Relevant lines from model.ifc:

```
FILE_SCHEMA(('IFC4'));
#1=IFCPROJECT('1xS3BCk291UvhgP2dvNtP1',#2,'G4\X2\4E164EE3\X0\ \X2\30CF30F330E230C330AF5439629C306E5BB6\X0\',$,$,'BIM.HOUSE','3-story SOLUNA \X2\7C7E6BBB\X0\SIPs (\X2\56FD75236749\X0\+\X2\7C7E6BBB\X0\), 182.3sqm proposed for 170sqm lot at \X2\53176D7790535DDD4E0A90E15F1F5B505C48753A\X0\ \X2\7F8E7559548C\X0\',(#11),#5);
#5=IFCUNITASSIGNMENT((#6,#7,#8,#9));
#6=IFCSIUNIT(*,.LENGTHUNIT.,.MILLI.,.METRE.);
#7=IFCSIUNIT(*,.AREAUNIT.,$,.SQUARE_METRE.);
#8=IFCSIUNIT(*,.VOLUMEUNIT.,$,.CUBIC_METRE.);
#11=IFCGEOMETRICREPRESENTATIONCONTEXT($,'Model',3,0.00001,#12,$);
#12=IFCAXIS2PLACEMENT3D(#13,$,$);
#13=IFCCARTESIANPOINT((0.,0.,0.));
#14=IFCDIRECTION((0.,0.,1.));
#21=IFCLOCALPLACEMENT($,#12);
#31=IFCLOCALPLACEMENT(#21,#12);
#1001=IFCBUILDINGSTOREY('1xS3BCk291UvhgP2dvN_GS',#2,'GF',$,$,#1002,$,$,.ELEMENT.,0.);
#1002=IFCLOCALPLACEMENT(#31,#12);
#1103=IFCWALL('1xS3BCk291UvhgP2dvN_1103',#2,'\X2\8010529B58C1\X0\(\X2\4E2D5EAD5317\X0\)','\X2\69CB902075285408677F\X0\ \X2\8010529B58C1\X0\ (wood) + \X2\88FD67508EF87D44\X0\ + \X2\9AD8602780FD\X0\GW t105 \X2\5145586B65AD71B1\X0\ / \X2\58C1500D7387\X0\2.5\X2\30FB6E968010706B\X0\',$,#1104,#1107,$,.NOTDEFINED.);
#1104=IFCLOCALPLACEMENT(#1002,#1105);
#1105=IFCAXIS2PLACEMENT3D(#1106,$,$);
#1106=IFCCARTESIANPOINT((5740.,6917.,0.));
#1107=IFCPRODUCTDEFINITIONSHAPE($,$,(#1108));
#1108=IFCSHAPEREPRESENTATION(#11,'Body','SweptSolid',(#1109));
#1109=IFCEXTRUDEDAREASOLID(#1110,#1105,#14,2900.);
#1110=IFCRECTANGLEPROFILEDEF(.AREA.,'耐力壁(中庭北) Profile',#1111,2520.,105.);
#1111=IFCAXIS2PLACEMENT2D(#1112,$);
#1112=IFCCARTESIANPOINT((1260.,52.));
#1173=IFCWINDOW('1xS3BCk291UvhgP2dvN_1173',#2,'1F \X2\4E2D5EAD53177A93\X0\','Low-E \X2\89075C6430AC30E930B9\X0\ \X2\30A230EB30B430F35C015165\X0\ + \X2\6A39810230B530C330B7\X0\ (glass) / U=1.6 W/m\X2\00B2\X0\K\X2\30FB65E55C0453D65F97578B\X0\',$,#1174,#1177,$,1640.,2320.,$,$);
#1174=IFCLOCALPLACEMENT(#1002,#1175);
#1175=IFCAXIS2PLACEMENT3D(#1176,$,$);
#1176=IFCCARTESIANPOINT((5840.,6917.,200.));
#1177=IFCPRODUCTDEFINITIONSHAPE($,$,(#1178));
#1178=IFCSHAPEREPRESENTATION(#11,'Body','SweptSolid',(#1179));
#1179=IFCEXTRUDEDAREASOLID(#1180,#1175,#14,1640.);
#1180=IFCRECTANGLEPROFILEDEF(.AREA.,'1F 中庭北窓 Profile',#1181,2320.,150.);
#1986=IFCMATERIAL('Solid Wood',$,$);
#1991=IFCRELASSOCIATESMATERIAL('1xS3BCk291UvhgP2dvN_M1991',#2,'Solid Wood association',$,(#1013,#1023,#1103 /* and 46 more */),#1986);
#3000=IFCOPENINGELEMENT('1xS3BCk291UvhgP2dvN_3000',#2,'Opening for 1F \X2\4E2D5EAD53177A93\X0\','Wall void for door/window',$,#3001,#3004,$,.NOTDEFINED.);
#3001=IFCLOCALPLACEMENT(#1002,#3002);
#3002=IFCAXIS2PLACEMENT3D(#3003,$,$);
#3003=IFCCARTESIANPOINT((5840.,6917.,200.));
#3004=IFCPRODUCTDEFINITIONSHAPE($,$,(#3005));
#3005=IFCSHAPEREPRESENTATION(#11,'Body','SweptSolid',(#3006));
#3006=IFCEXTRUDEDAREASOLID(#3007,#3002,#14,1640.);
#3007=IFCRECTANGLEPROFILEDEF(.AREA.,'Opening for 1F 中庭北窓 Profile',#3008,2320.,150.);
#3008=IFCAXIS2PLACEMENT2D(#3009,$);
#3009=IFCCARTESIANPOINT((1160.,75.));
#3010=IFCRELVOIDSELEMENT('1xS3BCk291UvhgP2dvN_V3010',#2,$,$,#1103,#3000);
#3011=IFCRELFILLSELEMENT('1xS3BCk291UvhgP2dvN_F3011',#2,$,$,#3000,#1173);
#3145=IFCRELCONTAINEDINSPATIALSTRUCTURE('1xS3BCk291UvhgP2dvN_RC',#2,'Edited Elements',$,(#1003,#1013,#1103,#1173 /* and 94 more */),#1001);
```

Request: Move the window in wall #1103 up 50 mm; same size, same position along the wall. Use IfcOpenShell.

```python
import numpy as np
import ifcopenshell
import ifcopenshell.api.geometry
import ifcopenshell.util.placement
import ifcopenshell.util.unit

model = ifcopenshell.open("model.ifc")
unit_scale = ifcopenshell.util.unit.calculate_unit_scale(model)

window = model.by_guid("1xS3BCk291UvhgP2dvN_1173")
opening = window.FillsVoids[0].RelatingOpeningElement
dz = 50.0

shift = np.array([0.0, 0.0, dz])
# The window is not placed relative to its opening, so move both.
for product in (opening, window):
    matrix = ifcopenshell.util.placement.get_local_placement(product.ObjectPlacement)
    matrix[:3, 3] += shift
    ifcopenshell.api.geometry.edit_object_placement(model, product=product, matrix=matrix, is_si=False)

print(f"moved by {dz * unit_scale:+.3f} m")

model.write("model_updated.ifc")
```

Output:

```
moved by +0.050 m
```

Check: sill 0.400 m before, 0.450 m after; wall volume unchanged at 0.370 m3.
